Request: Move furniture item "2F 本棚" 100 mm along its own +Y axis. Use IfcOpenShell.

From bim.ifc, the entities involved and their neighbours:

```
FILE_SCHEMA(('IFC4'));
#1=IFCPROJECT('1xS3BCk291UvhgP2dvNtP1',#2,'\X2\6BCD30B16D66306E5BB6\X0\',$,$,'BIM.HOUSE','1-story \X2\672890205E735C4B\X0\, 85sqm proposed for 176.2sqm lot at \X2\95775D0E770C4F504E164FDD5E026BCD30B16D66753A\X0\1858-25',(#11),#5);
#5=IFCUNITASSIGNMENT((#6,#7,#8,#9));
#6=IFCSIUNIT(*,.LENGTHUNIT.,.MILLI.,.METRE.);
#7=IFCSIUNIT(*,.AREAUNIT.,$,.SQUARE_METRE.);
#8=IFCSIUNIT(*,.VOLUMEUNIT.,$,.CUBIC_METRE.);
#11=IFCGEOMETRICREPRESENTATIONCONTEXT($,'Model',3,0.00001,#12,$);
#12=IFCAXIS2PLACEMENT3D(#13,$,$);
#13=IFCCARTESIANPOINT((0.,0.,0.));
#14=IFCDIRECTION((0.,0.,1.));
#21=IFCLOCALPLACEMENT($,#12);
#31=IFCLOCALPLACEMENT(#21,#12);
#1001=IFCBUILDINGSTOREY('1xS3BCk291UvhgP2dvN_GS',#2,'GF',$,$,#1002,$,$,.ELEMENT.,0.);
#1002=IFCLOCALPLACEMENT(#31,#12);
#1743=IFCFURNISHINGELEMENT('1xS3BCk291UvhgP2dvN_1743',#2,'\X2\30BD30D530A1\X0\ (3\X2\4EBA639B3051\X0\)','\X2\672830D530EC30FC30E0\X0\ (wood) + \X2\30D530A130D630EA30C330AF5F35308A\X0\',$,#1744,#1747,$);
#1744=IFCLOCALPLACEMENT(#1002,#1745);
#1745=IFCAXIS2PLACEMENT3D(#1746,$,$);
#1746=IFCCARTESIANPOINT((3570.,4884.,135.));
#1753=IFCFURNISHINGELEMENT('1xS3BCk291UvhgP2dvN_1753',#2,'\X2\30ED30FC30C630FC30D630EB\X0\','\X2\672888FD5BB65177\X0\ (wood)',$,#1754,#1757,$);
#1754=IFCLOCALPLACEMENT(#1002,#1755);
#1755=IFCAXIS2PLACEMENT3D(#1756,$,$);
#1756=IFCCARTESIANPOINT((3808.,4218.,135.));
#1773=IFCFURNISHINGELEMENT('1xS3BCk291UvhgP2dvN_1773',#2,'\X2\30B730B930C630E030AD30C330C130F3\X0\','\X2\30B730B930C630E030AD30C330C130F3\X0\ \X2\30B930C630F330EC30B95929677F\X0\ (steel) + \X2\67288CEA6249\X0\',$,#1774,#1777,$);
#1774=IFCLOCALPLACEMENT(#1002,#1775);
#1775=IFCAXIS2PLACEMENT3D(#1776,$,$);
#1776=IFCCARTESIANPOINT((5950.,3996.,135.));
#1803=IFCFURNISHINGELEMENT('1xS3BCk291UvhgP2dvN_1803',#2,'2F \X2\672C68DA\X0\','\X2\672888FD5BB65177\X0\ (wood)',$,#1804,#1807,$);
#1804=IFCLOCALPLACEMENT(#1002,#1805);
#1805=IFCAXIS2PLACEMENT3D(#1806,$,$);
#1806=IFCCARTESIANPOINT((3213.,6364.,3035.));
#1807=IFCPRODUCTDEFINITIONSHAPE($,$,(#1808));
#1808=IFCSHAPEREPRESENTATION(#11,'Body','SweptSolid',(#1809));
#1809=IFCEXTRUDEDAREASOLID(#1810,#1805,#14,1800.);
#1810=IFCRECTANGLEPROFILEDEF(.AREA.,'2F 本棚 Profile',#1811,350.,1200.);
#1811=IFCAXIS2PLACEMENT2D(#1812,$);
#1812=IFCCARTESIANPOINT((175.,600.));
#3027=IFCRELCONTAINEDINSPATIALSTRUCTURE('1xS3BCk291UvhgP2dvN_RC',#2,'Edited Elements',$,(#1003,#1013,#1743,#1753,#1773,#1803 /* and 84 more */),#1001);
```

```python
import ifcopenshell
import ifcopenshell.api.geometry
import ifcopenshell.util.placement

model = ifcopenshell.open("bim.ifc")

item = model.by_guid("1xS3BCk291UvhgP2dvN_1803")
matrix = ifcopenshell.util.placement.get_local_placement(item.ObjectPlacement)
matrix[:3, 3] += matrix[:3, 1] * 100.0
ifcopenshell.api.geometry.edit_object_placement(model, product=item, matrix=matrix, is_si=False)

print(ifcopenshell.util.placement.get_local_placement(item.ObjectPlacement).round(3) + 0.0)

model.write("bim_v2.ifc")
```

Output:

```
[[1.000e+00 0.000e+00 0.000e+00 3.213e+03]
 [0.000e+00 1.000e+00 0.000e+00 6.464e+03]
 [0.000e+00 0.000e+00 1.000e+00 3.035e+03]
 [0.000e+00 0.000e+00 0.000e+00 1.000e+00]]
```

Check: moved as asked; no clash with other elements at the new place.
